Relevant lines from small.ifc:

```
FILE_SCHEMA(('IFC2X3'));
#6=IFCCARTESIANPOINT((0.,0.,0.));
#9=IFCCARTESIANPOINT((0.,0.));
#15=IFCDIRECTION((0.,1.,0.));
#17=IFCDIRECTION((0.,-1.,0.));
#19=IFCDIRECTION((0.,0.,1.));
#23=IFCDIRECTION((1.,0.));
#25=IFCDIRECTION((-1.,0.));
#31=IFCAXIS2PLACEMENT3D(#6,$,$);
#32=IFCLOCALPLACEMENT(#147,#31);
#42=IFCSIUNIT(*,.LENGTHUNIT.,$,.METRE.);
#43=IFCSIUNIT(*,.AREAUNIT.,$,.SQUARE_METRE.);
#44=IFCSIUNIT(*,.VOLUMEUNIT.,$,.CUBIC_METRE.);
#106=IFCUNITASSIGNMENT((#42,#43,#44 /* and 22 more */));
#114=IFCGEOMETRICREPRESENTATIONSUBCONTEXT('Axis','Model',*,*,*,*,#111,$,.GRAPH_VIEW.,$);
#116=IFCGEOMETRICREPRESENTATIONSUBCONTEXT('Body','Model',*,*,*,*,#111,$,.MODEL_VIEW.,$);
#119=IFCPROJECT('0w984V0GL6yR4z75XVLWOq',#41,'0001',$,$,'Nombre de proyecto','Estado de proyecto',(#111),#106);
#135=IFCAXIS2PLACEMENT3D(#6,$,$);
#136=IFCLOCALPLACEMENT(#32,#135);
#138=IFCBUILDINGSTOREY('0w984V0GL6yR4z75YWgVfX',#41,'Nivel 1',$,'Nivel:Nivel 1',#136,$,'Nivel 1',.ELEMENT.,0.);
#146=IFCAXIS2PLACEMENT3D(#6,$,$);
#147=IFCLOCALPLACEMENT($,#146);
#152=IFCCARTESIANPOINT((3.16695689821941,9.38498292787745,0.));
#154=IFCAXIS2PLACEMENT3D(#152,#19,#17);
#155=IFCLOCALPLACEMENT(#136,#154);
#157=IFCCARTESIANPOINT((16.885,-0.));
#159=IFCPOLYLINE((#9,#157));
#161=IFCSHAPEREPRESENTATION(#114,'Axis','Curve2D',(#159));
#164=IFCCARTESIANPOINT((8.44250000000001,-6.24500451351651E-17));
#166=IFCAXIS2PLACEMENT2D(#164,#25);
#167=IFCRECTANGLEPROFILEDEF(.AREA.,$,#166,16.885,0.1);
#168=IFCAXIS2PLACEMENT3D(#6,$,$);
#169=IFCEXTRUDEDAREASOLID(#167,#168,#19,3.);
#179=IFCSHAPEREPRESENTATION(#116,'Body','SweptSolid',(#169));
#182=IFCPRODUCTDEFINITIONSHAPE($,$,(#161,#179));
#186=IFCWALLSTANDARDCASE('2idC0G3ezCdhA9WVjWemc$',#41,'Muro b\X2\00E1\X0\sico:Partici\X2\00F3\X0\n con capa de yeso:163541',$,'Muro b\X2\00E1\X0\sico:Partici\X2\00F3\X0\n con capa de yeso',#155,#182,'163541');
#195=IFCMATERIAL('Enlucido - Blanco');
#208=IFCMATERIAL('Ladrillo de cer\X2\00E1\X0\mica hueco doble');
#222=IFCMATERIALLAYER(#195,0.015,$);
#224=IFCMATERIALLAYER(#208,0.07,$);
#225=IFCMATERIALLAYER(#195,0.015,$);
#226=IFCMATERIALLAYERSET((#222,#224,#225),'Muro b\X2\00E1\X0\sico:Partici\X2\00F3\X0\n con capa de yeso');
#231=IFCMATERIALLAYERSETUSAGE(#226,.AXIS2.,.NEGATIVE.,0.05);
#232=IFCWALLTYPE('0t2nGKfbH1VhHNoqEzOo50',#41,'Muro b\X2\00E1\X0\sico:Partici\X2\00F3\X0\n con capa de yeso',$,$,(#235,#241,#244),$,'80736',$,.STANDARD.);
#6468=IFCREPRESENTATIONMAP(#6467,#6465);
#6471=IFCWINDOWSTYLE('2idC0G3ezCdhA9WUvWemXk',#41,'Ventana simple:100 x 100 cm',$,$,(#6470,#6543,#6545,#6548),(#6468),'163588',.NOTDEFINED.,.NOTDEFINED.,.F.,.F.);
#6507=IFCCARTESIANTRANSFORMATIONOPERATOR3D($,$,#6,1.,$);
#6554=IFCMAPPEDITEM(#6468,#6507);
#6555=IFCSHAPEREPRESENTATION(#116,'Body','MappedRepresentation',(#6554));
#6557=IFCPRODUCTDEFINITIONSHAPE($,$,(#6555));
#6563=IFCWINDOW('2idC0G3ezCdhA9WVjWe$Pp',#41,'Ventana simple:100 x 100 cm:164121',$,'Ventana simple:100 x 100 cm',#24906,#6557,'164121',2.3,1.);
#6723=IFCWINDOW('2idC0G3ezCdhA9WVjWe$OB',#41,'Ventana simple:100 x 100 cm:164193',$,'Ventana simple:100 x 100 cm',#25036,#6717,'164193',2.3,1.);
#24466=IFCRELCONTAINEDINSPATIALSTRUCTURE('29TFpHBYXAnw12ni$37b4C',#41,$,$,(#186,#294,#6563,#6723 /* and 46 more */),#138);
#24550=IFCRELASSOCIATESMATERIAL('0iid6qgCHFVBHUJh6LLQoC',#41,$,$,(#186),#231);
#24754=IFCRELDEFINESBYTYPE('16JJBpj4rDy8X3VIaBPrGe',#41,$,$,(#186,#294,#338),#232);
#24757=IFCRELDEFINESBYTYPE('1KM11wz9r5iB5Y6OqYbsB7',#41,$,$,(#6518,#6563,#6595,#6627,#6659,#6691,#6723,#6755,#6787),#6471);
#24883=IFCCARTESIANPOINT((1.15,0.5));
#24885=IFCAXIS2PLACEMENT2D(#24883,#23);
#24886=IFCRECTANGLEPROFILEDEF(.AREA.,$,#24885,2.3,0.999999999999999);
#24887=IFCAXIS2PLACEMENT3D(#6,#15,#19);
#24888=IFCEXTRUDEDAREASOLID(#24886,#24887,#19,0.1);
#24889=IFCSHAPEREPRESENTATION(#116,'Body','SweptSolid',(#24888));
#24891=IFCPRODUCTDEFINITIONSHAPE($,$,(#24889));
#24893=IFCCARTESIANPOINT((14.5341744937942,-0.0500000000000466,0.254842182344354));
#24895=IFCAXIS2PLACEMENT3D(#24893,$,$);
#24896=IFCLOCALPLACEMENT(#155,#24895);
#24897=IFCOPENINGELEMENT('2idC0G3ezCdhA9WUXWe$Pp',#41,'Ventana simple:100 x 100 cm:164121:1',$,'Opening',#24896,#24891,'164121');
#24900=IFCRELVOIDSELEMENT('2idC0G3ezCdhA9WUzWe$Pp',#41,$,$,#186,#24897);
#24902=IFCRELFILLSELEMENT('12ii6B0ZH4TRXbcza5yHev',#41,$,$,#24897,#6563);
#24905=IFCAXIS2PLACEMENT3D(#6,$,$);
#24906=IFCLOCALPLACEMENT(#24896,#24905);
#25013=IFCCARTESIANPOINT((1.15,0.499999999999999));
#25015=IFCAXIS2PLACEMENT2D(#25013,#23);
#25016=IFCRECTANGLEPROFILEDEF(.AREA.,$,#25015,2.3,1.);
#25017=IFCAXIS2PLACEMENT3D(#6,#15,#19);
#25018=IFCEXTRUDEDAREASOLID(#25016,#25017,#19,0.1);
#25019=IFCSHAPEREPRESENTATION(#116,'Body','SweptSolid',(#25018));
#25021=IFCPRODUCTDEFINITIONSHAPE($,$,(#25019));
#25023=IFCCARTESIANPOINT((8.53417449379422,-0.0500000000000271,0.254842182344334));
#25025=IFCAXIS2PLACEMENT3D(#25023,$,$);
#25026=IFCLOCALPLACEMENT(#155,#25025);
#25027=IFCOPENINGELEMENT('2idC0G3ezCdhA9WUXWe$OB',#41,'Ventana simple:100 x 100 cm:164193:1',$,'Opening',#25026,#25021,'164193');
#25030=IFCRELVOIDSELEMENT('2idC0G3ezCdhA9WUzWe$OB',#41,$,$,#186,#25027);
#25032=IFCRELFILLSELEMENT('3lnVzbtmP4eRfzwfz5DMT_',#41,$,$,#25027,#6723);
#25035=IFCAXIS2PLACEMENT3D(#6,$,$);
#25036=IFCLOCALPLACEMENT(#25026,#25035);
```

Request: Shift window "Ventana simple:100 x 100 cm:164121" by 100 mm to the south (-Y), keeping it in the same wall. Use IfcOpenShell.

```python
import ifcopenshell
import ifcopenshell.api.geometry
import ifcopenshell.util.placement

model = ifcopenshell.open("small.ifc")

window = model.by_guid("2idC0G3ezCdhA9WVjWe$Pp")
opening = window.FillsVoids[0].RelatingOpeningElement
wall = opening.VoidsElements[0].RelatingBuildingElement

wall_matrix = ifcopenshell.util.placement.get_local_placement(wall.ObjectPlacement)
shift = wall_matrix[:3, 0] * 0.1
before = ifcopenshell.util.placement.get_local_placement(window.ObjectPlacement)[:3, 3].copy()

# The window is placed relative to its opening, so it follows when the opening moves.
matrix = ifcopenshell.util.placement.get_local_placement(opening.ObjectPlacement)
matrix[:3, 3] += shift
ifcopenshell.api.geometry.edit_object_placement(
    model, product=opening, matrix=matrix, is_si=False, should_transform_children=True
)

after = ifcopenshell.util.placement.get_local_placement(window.ObjectPlacement)[:3, 3]
print("window moved by", (after - before).round(3) + 0.0)

model.write("small_rev.ifc")
```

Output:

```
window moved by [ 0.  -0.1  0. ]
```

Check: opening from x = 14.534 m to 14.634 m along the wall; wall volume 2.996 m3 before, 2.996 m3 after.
